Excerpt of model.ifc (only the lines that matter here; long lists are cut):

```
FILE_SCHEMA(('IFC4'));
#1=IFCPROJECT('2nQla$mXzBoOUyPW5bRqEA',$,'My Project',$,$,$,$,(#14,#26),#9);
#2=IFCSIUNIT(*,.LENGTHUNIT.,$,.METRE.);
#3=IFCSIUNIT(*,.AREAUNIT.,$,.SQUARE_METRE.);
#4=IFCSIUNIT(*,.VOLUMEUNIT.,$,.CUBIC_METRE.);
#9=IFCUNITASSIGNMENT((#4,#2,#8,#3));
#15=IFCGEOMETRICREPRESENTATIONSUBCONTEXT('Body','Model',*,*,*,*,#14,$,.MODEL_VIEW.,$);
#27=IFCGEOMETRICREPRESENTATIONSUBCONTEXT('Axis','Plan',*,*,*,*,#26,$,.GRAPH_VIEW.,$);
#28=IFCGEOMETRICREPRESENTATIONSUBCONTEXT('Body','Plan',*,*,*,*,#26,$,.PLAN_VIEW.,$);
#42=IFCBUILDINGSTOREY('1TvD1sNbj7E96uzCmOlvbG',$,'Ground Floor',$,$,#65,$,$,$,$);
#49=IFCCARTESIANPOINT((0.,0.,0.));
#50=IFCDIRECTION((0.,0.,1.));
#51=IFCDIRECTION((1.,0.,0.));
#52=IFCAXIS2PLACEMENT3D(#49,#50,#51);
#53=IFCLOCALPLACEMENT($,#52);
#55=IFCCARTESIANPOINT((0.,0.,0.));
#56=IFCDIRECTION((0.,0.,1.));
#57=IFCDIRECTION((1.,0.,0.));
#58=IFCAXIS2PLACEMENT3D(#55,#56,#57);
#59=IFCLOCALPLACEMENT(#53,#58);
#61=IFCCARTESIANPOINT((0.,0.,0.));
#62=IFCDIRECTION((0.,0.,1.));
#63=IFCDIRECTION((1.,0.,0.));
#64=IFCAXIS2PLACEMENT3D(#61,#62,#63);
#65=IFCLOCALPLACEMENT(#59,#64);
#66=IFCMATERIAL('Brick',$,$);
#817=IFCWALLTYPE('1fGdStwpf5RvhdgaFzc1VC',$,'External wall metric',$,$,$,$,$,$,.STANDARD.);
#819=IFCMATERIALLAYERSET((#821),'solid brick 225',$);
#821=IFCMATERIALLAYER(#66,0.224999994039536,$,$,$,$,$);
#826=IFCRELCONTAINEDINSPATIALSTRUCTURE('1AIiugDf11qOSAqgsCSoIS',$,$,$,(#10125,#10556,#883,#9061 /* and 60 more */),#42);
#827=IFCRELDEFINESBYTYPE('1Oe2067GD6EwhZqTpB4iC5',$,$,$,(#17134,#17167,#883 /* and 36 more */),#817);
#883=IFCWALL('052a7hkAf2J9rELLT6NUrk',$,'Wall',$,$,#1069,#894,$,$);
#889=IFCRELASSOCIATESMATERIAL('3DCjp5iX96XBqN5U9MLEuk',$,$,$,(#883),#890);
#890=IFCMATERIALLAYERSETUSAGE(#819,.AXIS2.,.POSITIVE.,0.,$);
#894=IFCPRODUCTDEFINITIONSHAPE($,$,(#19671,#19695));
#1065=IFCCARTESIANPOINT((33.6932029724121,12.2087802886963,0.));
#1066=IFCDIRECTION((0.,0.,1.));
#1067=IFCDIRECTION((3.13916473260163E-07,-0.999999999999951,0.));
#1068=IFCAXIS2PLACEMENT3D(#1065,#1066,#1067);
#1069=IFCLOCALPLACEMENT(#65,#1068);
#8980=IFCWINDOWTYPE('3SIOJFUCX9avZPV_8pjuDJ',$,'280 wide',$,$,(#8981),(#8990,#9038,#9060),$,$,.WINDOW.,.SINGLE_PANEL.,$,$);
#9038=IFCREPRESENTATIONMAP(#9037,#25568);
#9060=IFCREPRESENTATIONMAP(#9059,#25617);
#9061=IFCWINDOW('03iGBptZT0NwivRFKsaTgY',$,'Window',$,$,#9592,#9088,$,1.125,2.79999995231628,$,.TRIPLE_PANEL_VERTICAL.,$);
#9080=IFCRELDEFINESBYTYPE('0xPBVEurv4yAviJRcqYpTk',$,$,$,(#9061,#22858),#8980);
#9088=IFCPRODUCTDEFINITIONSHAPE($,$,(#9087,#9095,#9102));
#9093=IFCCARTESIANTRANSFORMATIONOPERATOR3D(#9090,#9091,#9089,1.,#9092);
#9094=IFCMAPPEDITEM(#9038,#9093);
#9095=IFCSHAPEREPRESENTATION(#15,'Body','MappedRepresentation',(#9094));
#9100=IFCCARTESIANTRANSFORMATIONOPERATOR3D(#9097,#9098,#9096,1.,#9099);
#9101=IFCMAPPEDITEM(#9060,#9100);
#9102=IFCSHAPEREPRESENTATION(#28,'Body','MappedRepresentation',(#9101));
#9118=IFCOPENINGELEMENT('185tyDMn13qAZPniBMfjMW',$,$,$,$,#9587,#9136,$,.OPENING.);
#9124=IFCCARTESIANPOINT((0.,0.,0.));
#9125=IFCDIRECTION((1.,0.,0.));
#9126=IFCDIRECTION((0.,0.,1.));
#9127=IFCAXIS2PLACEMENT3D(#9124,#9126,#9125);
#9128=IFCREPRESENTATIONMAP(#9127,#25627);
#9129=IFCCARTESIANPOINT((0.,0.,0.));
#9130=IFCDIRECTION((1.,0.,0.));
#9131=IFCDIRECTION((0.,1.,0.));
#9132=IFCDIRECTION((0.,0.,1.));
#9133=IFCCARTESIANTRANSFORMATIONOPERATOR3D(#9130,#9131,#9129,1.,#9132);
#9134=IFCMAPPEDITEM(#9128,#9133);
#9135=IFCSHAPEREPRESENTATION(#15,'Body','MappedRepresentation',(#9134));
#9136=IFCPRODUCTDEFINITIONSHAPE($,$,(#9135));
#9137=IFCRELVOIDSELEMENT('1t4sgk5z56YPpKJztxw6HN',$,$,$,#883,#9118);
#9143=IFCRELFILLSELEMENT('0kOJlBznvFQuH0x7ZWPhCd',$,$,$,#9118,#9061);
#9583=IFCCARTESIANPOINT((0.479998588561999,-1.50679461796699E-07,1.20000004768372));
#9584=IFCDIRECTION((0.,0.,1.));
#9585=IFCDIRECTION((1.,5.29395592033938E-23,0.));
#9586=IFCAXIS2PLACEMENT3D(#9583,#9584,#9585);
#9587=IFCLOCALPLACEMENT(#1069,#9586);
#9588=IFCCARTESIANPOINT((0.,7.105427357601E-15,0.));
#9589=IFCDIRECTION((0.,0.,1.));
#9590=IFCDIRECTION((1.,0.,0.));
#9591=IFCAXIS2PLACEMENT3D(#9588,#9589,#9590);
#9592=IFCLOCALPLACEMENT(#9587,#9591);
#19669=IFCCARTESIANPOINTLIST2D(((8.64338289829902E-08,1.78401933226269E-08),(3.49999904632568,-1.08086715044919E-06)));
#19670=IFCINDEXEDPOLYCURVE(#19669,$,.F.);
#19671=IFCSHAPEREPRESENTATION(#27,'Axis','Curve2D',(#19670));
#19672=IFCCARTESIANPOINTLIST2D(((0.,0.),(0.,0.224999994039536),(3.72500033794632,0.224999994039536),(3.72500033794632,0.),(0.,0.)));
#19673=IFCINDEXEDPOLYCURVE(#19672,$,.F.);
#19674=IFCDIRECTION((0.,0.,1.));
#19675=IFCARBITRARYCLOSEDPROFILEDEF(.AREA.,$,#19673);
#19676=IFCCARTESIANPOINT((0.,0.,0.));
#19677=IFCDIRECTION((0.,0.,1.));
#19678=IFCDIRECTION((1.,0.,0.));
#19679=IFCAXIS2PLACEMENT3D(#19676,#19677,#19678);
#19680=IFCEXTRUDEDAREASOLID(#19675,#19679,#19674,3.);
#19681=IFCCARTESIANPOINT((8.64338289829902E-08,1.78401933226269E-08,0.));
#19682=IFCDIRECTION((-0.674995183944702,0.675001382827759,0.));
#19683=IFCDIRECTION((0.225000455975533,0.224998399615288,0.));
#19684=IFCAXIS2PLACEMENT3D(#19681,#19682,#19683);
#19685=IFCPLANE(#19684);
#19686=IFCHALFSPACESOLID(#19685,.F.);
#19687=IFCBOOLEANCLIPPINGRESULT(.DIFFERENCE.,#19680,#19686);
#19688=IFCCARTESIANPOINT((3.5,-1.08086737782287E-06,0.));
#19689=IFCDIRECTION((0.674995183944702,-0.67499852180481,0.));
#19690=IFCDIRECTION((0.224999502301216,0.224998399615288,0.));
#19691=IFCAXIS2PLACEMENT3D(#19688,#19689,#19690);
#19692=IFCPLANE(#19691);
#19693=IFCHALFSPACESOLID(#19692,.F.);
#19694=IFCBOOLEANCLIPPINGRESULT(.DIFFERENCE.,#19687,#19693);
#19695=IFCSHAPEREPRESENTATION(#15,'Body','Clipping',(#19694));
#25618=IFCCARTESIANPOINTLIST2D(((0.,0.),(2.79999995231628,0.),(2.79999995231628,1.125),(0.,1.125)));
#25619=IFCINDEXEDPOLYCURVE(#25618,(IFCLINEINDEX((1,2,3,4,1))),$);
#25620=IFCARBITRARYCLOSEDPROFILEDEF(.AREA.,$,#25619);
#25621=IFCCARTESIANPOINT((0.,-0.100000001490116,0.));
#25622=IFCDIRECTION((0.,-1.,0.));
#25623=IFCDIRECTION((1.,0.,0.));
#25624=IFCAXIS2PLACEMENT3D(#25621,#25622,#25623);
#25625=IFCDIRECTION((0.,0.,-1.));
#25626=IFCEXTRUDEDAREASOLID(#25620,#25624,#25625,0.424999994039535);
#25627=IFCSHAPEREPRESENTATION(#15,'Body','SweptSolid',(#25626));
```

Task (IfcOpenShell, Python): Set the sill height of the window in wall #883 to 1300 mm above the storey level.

```python
import numpy as np
import ifcopenshell
import ifcopenshell.api.geometry
import ifcopenshell.geom
import ifcopenshell.util.element
import ifcopenshell.util.placement
import ifcopenshell.util.shape
import ifcopenshell.util.unit

model = ifcopenshell.open("model.ifc")
unit_scale = ifcopenshell.util.unit.calculate_unit_scale(model)

window = model.by_guid("03iGBptZT0NwivRFKsaTgY")
opening = window.FillsVoids[0].RelatingOpeningElement
storey = ifcopenshell.util.element.get_container(window, ifc_class="IfcBuildingStorey")
level = ifcopenshell.util.placement.get_local_placement(storey.ObjectPlacement)[2, 3]

# The opening's origin need not be at the sill, so measure its lowest point.
shape = ifcopenshell.geom.create_shape(ifcopenshell.geom.settings(), opening)
bottom = ifcopenshell.util.shape.get_shape_bottom_elevation(shape, shape.geometry) / unit_scale
dz = level + 1.3 - bottom

shift = np.array([0.0, 0.0, dz])
# The window is placed relative to its opening, so it follows when the opening moves.
matrix = ifcopenshell.util.placement.get_local_placement(opening.ObjectPlacement)
matrix[:3, 3] += shift
ifcopenshell.api.geometry.edit_object_placement(
    model, product=opening, matrix=matrix, is_si=False, should_transform_children=True
)

print(f"moved by {dz * unit_scale:+.3f} m")

model.write("model_rev.ifc")
```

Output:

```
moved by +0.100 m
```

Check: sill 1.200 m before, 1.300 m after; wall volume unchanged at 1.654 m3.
